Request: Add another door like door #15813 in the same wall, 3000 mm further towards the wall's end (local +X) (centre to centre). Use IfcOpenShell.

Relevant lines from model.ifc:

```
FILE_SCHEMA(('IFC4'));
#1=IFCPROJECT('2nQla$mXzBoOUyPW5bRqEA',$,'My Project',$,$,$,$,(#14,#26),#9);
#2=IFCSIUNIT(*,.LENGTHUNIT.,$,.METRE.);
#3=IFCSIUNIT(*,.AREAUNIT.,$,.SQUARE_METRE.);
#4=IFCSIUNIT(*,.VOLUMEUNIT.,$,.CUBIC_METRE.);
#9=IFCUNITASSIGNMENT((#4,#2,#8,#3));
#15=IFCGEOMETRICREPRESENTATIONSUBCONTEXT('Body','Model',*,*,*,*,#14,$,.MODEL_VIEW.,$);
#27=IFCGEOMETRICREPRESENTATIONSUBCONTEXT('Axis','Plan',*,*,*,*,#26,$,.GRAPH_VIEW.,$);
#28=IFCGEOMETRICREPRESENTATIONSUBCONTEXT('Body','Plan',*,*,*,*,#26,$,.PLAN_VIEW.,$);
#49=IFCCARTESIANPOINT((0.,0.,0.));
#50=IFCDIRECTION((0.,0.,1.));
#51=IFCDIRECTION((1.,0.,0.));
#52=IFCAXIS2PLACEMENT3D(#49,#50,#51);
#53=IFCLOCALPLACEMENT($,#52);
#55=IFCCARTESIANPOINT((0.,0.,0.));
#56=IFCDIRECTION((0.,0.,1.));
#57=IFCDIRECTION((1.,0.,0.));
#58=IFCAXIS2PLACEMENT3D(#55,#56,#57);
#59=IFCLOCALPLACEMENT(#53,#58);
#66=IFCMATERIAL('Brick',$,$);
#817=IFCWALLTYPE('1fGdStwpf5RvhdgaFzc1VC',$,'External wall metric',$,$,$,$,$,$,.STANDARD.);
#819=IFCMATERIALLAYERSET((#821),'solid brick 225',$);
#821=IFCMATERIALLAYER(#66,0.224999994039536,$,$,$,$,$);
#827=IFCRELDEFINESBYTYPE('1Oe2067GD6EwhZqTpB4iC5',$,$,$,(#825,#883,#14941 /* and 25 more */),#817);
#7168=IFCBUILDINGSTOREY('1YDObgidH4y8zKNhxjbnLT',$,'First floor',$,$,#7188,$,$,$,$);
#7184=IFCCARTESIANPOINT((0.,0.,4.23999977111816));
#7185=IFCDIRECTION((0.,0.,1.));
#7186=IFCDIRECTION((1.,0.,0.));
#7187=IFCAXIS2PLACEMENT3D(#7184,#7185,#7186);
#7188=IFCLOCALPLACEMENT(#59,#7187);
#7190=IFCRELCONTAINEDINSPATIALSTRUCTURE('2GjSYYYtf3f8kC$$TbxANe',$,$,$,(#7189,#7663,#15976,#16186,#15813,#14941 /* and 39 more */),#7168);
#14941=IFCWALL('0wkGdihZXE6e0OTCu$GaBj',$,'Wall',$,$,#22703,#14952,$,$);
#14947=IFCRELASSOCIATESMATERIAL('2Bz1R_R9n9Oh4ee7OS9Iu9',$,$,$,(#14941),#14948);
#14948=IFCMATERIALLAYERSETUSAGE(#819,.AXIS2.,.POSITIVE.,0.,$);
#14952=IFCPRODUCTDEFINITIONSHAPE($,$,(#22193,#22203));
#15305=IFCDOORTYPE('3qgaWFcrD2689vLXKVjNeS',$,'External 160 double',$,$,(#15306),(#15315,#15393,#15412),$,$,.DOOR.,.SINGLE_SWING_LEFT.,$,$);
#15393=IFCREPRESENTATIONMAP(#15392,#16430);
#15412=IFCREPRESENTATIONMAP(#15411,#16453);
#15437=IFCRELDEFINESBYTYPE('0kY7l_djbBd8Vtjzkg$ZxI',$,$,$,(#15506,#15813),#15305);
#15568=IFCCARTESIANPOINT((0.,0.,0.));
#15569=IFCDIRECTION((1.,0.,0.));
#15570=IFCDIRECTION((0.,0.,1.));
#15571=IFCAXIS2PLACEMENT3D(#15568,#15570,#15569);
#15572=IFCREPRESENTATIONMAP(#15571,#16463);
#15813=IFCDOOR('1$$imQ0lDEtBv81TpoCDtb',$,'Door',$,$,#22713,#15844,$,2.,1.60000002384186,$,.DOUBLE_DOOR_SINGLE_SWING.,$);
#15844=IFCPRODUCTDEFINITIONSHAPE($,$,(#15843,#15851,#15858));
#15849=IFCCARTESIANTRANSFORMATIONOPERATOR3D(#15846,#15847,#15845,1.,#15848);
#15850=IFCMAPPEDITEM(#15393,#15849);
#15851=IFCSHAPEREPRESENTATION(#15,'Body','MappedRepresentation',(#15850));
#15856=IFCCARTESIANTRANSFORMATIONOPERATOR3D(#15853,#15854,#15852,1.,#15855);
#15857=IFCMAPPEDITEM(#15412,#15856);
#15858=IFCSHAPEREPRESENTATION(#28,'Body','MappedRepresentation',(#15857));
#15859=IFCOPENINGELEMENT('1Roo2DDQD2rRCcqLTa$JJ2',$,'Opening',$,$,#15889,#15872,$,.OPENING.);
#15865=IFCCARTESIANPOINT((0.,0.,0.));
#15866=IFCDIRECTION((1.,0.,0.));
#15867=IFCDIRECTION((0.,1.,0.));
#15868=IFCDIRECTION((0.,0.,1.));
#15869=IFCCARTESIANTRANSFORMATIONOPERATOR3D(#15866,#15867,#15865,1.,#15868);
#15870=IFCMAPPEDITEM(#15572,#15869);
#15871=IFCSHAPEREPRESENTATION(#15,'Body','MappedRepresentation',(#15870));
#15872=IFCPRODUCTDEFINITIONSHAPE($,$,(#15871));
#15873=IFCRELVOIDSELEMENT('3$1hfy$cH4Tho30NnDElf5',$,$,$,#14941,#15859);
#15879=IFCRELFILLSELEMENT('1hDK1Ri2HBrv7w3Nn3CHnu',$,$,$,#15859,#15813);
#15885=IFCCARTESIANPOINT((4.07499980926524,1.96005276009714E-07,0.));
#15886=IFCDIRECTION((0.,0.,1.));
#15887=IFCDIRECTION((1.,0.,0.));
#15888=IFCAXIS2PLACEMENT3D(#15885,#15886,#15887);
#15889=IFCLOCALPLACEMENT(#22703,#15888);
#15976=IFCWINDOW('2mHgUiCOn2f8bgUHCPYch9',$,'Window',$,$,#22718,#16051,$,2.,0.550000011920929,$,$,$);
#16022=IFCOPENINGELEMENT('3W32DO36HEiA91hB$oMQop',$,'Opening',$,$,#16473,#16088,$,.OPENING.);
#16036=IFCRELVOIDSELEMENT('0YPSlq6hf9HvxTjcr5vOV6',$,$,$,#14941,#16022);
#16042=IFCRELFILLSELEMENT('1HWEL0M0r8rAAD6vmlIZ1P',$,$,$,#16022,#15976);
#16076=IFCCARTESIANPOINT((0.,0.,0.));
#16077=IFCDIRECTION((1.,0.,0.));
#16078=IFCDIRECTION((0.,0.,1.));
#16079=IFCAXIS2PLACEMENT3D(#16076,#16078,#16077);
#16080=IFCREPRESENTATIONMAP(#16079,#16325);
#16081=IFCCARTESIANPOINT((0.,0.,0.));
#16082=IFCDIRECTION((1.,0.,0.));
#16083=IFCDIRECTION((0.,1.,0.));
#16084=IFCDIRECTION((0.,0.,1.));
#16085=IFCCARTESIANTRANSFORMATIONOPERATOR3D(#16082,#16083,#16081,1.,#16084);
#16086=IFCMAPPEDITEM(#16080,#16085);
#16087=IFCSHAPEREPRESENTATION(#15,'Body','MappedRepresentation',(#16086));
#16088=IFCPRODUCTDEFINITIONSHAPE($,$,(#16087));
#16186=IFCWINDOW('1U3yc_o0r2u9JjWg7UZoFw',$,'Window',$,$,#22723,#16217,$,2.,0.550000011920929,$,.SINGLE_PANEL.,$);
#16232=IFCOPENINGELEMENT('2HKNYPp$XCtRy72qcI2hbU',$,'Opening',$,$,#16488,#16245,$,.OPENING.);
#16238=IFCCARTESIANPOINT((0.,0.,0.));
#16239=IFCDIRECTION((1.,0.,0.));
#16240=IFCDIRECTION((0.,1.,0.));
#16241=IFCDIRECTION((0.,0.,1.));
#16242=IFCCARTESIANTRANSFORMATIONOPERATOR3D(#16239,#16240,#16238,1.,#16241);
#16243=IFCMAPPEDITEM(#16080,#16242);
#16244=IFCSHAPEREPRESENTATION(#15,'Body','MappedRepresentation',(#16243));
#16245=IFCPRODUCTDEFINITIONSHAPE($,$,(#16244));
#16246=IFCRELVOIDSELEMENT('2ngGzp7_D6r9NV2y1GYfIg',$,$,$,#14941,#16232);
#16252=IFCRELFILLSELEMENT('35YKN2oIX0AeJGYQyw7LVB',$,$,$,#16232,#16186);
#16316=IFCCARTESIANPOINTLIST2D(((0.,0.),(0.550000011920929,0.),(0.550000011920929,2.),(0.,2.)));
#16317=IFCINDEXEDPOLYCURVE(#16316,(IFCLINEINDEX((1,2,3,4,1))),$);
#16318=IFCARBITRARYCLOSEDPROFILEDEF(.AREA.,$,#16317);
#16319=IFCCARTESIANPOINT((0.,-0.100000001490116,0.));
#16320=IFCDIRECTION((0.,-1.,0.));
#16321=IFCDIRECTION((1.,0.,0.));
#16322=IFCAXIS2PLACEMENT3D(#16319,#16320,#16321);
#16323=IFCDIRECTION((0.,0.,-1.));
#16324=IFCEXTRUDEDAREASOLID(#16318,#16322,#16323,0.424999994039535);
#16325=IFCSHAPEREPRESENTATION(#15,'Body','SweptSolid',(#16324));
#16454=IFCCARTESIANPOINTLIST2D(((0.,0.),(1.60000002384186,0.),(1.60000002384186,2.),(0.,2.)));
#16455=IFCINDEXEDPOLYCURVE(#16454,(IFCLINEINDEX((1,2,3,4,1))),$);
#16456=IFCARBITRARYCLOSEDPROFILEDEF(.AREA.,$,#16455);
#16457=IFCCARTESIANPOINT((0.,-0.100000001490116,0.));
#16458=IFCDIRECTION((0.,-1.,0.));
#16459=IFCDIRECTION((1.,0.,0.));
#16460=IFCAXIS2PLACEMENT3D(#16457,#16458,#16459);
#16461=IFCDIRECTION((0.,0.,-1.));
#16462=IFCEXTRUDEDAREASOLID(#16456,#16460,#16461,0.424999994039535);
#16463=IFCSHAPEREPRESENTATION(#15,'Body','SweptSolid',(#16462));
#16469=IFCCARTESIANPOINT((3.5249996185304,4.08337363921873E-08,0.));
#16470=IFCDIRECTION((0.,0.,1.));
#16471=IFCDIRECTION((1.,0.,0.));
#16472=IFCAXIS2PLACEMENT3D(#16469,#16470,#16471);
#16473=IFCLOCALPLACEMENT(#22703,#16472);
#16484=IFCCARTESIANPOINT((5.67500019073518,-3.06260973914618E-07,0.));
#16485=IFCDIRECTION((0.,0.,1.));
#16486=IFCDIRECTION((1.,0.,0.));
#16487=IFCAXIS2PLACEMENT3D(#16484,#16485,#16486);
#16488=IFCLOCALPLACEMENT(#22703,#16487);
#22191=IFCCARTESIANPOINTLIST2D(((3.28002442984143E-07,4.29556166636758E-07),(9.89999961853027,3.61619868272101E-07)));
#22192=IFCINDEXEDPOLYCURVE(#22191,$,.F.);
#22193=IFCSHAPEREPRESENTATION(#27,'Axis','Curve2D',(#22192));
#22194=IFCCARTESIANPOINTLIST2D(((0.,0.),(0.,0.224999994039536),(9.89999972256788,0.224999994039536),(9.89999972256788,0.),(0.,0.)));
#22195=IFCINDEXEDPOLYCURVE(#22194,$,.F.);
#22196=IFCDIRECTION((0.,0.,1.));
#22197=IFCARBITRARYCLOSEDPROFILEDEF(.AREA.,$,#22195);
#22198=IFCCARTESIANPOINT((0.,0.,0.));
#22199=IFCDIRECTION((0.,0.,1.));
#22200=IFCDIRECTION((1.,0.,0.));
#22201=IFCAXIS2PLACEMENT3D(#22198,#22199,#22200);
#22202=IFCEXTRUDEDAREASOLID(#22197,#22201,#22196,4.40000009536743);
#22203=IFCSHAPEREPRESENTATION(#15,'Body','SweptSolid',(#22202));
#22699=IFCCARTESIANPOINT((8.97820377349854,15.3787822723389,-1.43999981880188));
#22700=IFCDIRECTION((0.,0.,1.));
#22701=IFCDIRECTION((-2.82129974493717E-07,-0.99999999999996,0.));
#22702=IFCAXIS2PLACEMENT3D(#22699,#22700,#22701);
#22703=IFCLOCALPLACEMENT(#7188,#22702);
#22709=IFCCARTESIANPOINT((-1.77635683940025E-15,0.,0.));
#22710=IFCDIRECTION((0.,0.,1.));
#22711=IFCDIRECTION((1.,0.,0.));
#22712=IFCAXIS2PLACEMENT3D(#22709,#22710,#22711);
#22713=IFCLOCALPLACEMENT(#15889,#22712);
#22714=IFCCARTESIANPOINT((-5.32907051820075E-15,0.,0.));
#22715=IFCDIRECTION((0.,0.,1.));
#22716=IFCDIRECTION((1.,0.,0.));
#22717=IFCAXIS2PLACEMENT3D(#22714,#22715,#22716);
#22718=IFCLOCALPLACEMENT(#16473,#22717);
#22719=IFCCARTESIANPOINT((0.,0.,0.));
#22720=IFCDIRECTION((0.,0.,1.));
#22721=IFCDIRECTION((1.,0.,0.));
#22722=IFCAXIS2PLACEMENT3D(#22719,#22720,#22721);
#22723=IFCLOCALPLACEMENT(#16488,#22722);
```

```python
import ifcopenshell
import ifcopenshell.api.feature
import ifcopenshell.api.geometry
import ifcopenshell.api.root
import ifcopenshell.geom
import ifcopenshell.util.element
import ifcopenshell.util.placement
import ifcopenshell.util.shape

model = ifcopenshell.open("model.ifc")
settings = ifcopenshell.geom.settings()


def volume(element):
    """Net volume in cubic metres, openings subtracted."""
    shape = ifcopenshell.geom.create_shape(settings, element)
    return ifcopenshell.util.shape.get_volume(shape.geometry)


door = model.by_guid("1$$imQ0lDEtBv81TpoCDtb")
opening = door.FillsVoids[0].RelatingOpeningElement
wall = opening.VoidsElements[0].RelatingBuildingElement
before = volume(wall)
shift = ifcopenshell.util.placement.get_local_placement(wall.ObjectPlacement)[:3, 0] * 3.0

# copy_class copies the void relationship, type, container and properties, but no geometry.
new_opening = ifcopenshell.api.root.copy_class(model, product=opening)
new_opening.Representation = ifcopenshell.util.element.copy_deep(
    model, opening.Representation, exclude=["IfcGeometricRepresentationContext", "IfcRepresentationMap"]
)
new_door = ifcopenshell.api.root.copy_class(model, product=door)
new_door.Representation = ifcopenshell.util.element.copy_deep(
    model, door.Representation, exclude=["IfcGeometricRepresentationContext", "IfcRepresentationMap"]
)
ifcopenshell.api.feature.add_filling(model, opening=new_opening, element=new_door)

for old, new in ((opening, new_opening), (door, new_door)):
    matrix = ifcopenshell.util.placement.get_local_placement(old.ObjectPlacement)
    matrix[:3, 3] += shift
    ifcopenshell.api.geometry.edit_object_placement(model, product=new, matrix=matrix, is_si=False)

after = volume(wall)

print(f"wall volume {before:.3f} -> {after:.3f} m3")

model.write("model_v2.ifc")
```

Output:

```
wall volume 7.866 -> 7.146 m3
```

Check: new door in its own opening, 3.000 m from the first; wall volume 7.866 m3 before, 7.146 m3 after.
